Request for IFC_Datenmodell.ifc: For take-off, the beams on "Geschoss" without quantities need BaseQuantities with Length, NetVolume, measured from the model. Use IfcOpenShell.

First a look at what the model holds.

```python
import ifcopenshell
import ifcopenshell.util.element
import ifcopenshell.util.unit

model = ifcopenshell.open("IFC_Datenmodell.ifc")
print(model.schema)
for unit_type in ("LENGTHUNIT", "AREAUNIT", "VOLUMEUNIT"):
    print(unit_type, ifcopenshell.util.unit.calculate_unit_scale(model, unit_type))
storey = next(s for s in model.by_type("IfcBuildingStorey") if s.Name == "Geschoss")
beams = [e for e in ifcopenshell.util.element.get_decomposition(storey) if e.is_a("IfcBeam")]
for e in sorted(beams, key=lambda e: e.id()):
    print(e.id(), e.is_a(), e.Name, list(ifcopenshell.util.element.get_psets(e, qtos_only=True)), sep=" | ")
```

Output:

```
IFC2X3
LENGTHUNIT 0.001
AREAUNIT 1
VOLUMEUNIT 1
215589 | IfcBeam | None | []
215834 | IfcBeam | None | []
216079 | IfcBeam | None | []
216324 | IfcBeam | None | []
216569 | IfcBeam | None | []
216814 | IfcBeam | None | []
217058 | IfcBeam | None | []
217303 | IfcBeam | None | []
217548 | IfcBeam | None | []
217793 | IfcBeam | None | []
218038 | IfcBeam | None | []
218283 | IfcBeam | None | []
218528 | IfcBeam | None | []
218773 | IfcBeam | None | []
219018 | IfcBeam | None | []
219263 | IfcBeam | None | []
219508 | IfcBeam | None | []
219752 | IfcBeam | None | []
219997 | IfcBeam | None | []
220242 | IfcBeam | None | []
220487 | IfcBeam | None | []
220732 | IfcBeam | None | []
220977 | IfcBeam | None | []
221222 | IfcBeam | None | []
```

```python
import ifcopenshell
import ifcopenshell.api.pset
import ifcopenshell.geom
import ifcopenshell.util.element
import ifcopenshell.util.shape
import ifcopenshell.util.unit

model = ifcopenshell.open("IFC_Datenmodell.ifc")
unit_scale = ifcopenshell.util.unit.calculate_unit_scale(model)
volume_scale = ifcopenshell.util.unit.calculate_unit_scale(model, "VOLUMEUNIT")
settings = ifcopenshell.geom.settings()

storey = next(s for s in model.by_type("IfcBuildingStorey") if s.Name == "Geschoss")
beams = [e for e in ifcopenshell.util.element.get_decomposition(storey) if e.is_a("IfcBeam")]

for e in sorted(beams, key=lambda e: e.id()):
    if ifcopenshell.util.element.get_psets(e, qtos_only=True, should_inherit=False):
        continue
    # Geometry comes back in metres, in the element's own axes.
    shape = ifcopenshell.geom.create_shape(settings, e)
    values = {
        "Length": ifcopenshell.util.shape.get_max_xyz(shape.geometry) / unit_scale,
        "NetVolume": ifcopenshell.util.shape.get_volume(shape.geometry) / volume_scale,
    }
    qto = ifcopenshell.api.pset.add_qto(model, product=e, name="BaseQuantities")
    ifcopenshell.api.pset.edit_qto(model, qto=qto, properties=values)
    print(e.id(), {k: round(v, 3) for k, v in values.items()})

model.write("IFC_Datenmodell-out.ifc")
```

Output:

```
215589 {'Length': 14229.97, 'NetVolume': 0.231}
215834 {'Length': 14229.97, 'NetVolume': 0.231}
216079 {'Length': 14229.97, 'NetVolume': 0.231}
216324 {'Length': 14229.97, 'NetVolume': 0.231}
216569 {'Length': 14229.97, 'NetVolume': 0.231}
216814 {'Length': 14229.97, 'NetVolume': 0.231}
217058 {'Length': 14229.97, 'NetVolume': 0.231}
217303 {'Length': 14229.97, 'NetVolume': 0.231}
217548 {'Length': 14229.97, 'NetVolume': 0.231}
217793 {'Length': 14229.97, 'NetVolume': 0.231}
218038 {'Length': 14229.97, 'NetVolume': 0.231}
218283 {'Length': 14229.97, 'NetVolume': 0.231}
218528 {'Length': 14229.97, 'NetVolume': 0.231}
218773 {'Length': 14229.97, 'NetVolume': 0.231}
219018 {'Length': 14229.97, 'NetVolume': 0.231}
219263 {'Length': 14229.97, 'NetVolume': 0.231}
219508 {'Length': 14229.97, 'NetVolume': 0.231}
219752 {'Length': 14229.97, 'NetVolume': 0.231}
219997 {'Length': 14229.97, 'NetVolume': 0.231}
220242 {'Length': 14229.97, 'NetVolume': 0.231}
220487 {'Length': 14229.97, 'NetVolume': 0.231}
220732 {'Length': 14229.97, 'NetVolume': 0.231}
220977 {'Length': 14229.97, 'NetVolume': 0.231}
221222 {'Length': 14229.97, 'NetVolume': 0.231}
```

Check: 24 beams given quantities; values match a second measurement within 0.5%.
